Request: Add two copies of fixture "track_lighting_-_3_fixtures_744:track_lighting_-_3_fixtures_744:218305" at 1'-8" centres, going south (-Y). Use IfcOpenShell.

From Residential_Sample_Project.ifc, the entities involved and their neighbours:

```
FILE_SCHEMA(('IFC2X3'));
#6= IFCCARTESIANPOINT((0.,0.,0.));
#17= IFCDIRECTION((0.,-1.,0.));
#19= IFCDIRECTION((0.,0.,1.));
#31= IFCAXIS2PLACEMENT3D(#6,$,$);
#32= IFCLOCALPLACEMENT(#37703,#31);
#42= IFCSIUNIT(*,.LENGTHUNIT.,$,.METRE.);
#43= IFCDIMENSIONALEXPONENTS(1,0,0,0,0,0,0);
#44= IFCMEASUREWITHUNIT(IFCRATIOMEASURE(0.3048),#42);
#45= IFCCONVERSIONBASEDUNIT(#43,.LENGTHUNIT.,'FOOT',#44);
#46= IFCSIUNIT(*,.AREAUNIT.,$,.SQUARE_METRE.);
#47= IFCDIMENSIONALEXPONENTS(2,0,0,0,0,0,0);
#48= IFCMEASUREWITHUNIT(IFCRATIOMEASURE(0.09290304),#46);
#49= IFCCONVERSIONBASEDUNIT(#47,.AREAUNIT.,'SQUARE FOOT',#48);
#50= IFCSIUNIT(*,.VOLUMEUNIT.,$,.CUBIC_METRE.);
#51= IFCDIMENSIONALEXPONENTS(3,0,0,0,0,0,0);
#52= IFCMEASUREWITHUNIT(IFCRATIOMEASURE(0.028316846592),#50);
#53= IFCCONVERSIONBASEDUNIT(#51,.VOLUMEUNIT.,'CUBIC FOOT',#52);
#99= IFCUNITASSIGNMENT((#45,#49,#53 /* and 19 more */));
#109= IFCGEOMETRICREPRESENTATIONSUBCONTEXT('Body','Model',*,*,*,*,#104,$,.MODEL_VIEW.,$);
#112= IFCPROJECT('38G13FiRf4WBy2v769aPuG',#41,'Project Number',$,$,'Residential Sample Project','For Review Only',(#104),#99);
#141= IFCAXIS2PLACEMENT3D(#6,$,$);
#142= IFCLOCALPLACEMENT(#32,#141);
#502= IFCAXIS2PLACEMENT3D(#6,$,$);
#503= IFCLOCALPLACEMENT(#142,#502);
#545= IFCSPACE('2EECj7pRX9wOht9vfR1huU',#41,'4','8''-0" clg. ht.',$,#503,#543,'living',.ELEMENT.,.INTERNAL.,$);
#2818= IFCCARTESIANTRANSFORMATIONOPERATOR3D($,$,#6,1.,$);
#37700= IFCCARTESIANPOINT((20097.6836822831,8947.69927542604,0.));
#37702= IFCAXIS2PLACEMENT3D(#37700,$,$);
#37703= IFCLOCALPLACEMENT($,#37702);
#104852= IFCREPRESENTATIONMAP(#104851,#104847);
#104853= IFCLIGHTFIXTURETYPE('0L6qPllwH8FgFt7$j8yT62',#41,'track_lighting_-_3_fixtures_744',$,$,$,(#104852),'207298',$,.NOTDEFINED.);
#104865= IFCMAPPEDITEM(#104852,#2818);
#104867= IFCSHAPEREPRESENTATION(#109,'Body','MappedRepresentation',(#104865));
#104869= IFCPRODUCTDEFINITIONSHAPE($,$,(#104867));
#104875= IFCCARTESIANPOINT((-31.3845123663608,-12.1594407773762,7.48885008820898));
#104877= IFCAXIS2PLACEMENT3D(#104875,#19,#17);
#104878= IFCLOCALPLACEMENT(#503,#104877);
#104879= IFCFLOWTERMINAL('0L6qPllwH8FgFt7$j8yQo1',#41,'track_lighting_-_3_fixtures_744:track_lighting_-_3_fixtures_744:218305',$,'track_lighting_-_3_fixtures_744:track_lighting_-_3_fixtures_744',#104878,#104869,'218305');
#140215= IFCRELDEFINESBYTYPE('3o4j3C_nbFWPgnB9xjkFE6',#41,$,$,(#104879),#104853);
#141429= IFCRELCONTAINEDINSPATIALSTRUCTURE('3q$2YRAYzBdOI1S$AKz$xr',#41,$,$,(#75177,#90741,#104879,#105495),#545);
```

```python
import numpy as np
import ifcopenshell
import ifcopenshell.api.geometry
import ifcopenshell.api.root
import ifcopenshell.util.element
import ifcopenshell.util.placement
import ifcopenshell.util.unit

model = ifcopenshell.open("Residential_Sample_Project.ifc")
unit_scale = ifcopenshell.util.unit.calculate_unit_scale(model)


def reuse_history(source, copy):
    """copy_class also copies each property set's owner history, people and application; keep the originals."""
    for rel in copy.IsDefinedBy:
        if rel.is_a("IfcRelDefinesByProperties") and (history := rel.RelatingPropertyDefinition.OwnerHistory):
            rel.RelatingPropertyDefinition.OwnerHistory = source.OwnerHistory
            ifcopenshell.util.element.remove_deep2(model, history)


source = model.by_id(104879)
base = ifcopenshell.util.placement.get_local_placement(source.ObjectPlacement)
step = np.array([0.0, -1.0, 0.0]) * 20 * 0.0254 / unit_scale

for i in range(1, 3):
    copy = ifcopenshell.api.root.copy_class(model, product=source)
    copy.Representation = ifcopenshell.util.element.copy_deep(
        model, source.Representation, exclude=["IfcGeometricRepresentationContext", "IfcRepresentationMap"]
    )
    copy.Name = "track_lighting_-_3_fixtures_744:track_lighting_-_3_fixtures_744"
    copy.Tag = None
    reuse_history(source, copy)
    matrix = base.copy()
    matrix[:3, 3] += i * step
    print("added at", matrix[:3, 3].round(3) + 0.0)
    ifcopenshell.api.geometry.edit_object_placement(model, product=copy, matrix=matrix, is_si=False)

model.write("Residential_Sample_Project_edited.ifc")
```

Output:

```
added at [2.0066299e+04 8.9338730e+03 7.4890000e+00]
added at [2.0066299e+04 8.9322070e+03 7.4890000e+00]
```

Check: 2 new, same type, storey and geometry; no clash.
